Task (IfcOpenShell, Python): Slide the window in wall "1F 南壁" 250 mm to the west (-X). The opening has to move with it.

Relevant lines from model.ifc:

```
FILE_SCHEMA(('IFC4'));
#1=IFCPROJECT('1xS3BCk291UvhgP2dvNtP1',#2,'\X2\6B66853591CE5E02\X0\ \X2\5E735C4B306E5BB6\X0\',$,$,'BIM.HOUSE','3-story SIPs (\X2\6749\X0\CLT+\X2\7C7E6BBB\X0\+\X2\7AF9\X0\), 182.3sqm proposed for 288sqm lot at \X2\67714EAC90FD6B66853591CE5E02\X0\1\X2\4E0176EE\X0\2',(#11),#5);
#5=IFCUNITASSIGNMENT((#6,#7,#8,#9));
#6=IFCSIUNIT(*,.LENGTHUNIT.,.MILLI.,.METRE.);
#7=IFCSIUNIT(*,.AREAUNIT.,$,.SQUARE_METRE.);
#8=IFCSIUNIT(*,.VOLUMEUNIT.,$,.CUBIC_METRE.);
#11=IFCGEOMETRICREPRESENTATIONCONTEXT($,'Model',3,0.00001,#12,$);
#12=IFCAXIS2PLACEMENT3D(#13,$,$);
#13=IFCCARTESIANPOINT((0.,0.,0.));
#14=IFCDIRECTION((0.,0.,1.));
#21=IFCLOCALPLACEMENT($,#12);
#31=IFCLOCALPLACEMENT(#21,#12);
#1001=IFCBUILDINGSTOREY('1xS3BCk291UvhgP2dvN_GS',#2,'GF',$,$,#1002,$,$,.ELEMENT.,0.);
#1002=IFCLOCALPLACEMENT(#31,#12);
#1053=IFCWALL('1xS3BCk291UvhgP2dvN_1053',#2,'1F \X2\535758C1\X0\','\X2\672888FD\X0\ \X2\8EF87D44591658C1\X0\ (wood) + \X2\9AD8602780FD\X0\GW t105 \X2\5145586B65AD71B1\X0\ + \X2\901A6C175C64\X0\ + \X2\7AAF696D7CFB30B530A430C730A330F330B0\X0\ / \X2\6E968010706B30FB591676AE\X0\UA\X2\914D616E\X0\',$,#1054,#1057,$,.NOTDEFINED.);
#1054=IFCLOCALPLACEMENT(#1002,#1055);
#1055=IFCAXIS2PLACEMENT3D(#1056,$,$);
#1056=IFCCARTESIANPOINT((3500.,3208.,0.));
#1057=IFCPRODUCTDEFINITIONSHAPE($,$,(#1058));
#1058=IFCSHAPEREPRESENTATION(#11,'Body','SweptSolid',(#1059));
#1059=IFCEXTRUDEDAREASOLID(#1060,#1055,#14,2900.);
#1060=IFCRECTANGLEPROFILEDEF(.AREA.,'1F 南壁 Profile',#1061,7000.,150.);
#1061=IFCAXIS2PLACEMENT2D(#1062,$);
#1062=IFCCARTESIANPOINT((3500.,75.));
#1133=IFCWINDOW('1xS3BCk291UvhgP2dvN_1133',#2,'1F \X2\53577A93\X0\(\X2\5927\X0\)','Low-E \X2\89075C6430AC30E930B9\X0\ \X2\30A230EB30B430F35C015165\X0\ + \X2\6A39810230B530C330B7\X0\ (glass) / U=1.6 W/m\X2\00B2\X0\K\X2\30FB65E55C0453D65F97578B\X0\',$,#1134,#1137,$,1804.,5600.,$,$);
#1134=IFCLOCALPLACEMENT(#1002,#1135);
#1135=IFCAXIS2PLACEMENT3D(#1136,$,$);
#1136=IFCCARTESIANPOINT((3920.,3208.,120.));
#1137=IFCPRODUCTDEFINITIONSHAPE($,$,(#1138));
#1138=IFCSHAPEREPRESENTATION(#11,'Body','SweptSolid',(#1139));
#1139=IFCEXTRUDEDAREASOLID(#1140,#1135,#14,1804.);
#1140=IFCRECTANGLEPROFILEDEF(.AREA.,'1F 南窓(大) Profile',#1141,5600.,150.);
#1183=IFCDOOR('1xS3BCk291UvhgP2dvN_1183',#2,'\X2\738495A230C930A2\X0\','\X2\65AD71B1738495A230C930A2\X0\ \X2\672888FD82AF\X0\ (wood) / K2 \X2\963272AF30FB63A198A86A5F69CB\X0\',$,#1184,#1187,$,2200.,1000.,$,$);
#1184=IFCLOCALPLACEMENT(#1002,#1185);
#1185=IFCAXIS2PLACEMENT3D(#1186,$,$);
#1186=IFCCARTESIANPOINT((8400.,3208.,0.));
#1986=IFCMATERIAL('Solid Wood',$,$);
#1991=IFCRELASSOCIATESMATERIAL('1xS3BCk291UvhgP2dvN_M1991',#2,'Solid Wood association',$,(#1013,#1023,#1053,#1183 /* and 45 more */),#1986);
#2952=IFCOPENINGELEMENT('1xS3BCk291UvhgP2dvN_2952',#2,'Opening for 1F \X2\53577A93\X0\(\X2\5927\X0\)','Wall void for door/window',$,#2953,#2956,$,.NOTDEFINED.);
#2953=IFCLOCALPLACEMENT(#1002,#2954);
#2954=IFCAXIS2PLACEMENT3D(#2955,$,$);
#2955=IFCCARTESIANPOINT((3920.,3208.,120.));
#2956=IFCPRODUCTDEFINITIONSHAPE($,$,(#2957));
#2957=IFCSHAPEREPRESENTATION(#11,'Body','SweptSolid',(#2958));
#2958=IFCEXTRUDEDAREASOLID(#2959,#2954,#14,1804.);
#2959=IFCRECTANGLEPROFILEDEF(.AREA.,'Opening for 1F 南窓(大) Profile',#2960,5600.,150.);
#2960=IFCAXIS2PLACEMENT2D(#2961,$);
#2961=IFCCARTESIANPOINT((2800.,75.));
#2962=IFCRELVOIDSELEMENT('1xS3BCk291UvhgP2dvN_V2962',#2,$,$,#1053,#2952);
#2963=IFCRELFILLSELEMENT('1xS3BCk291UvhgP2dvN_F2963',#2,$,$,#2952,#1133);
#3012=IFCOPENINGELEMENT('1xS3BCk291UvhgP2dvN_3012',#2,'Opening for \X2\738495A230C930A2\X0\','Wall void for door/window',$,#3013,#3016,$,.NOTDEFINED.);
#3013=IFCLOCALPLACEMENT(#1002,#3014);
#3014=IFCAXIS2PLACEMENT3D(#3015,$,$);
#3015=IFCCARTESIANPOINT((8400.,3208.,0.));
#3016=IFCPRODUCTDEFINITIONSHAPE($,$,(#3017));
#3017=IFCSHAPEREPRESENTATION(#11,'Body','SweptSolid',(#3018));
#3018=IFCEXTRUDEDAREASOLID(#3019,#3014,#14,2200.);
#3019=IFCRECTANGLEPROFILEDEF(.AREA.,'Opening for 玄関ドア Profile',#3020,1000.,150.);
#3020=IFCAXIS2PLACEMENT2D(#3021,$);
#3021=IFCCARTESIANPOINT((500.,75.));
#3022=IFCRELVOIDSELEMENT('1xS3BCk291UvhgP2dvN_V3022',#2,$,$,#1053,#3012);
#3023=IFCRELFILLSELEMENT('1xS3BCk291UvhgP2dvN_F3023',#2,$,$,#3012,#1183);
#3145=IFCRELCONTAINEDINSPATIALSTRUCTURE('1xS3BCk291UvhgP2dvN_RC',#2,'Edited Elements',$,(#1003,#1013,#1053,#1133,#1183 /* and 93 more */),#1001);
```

```python
import ifcopenshell
import ifcopenshell.api.geometry
import ifcopenshell.util.placement
import ifcopenshell.util.unit

model = ifcopenshell.open("model.ifc")
unit_scale = ifcopenshell.util.unit.calculate_unit_scale(model)

window = model.by_guid("1xS3BCk291UvhgP2dvN_1133")
opening = window.FillsVoids[0].RelatingOpeningElement
wall = opening.VoidsElements[0].RelatingBuildingElement

wall_matrix = ifcopenshell.util.placement.get_local_placement(wall.ObjectPlacement)
shift = wall_matrix[:3, 0] * -0.25 / unit_scale
before = ifcopenshell.util.placement.get_local_placement(window.ObjectPlacement)[:3, 3].copy()

# The window is not placed relative to its opening, so move both.
for product in (opening, window):
    matrix = ifcopenshell.util.placement.get_local_placement(product.ObjectPlacement)
    matrix[:3, 3] += shift
    ifcopenshell.api.geometry.edit_object_placement(model, product=product, matrix=matrix, is_si=False)

after = ifcopenshell.util.placement.get_local_placement(window.ObjectPlacement)[:3, 3]
print("window moved by", (after - before).round(3) + 0.0)

model.write("model-out.ifc")
```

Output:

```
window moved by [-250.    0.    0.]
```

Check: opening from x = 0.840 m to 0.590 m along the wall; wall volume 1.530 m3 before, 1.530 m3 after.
